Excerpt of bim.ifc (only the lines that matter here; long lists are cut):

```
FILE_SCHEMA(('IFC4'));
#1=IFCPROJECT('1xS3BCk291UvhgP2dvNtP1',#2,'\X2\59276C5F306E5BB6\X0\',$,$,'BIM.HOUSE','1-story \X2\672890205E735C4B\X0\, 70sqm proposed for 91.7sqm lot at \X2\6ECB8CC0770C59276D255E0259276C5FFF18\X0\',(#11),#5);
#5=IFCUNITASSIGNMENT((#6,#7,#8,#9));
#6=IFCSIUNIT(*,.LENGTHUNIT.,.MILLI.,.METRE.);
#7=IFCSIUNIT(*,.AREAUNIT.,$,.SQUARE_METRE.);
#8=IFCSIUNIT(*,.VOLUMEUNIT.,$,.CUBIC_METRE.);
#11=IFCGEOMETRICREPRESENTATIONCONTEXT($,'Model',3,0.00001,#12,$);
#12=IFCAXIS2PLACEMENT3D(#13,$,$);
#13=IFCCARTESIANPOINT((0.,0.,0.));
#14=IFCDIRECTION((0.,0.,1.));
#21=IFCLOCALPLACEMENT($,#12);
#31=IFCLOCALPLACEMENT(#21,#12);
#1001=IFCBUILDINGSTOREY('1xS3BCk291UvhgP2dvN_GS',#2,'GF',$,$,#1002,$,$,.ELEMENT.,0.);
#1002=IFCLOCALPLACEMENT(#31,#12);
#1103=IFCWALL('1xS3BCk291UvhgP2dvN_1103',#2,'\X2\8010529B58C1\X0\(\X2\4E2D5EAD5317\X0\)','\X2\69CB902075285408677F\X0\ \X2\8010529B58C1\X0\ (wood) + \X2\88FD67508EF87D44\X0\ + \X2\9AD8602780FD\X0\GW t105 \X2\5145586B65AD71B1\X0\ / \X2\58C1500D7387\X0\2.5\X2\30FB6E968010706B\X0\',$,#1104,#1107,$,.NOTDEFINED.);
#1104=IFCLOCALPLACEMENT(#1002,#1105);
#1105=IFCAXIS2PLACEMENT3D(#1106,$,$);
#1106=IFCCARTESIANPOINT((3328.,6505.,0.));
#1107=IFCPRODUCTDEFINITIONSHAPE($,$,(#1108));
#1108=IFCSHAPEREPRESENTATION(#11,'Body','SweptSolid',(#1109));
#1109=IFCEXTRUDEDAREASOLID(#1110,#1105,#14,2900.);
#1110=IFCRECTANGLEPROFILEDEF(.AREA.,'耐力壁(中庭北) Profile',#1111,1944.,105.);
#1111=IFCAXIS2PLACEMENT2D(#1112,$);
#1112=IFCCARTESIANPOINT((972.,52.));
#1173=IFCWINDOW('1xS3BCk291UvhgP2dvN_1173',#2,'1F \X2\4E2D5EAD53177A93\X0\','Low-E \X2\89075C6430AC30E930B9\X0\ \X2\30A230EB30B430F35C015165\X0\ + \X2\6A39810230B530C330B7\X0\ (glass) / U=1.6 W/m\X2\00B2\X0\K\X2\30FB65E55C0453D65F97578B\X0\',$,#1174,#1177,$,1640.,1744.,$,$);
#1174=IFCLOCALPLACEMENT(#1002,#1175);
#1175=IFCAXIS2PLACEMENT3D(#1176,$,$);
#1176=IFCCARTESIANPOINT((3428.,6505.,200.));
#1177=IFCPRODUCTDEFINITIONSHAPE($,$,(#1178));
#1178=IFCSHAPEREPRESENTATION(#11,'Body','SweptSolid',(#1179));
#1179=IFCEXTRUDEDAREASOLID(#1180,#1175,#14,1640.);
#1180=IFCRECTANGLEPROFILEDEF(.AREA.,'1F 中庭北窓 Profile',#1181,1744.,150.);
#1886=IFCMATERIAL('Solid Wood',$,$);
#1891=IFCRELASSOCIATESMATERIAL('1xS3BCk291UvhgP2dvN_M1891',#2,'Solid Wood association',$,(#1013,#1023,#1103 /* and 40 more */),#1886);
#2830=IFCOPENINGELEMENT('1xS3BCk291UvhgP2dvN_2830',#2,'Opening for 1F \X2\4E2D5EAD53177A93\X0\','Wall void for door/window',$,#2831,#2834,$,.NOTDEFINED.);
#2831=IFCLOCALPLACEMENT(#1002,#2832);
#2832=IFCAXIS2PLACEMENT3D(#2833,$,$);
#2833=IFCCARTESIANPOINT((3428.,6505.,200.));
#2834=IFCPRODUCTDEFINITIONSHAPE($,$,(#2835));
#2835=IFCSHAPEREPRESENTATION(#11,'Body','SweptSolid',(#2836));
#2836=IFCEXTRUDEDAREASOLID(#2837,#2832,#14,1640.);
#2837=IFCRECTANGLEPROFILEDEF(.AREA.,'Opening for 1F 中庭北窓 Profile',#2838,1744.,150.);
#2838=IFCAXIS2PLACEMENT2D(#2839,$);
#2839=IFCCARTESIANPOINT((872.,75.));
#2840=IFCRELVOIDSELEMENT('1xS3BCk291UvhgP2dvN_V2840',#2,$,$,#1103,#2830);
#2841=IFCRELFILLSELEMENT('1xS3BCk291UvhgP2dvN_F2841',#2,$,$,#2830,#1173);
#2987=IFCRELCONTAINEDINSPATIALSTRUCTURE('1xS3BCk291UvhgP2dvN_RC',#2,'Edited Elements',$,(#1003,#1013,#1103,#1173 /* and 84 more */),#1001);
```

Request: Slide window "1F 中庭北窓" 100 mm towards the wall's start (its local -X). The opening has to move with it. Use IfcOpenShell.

```python
import ifcopenshell
import ifcopenshell.api.geometry
import ifcopenshell.util.placement
import ifcopenshell.util.unit

model = ifcopenshell.open("bim.ifc")
unit_scale = ifcopenshell.util.unit.calculate_unit_scale(model)

window = model.by_id(1173)
opening = window.FillsVoids[0].RelatingOpeningElement
wall = opening.VoidsElements[0].RelatingBuildingElement

wall_matrix = ifcopenshell.util.placement.get_local_placement(wall.ObjectPlacement)
shift = wall_matrix[:3, 0] * -0.1 / unit_scale
before = ifcopenshell.util.placement.get_local_placement(window.ObjectPlacement)[:3, 3].copy()

# The window is not placed relative to its opening, so move both.
for product in (opening, window):
    matrix = ifcopenshell.util.placement.get_local_placement(product.ObjectPlacement)
    matrix[:3, 3] += shift
    ifcopenshell.api.geometry.edit_object_placement(model, product=product, matrix=matrix, is_si=False)

after = ifcopenshell.util.placement.get_local_placement(window.ObjectPlacement)[:3, 3]
print("window moved by", (after - before).round(3) + 0.0)

model.write("bim_v2.ifc")
```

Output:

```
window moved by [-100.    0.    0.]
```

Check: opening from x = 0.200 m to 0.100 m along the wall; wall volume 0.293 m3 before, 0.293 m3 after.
